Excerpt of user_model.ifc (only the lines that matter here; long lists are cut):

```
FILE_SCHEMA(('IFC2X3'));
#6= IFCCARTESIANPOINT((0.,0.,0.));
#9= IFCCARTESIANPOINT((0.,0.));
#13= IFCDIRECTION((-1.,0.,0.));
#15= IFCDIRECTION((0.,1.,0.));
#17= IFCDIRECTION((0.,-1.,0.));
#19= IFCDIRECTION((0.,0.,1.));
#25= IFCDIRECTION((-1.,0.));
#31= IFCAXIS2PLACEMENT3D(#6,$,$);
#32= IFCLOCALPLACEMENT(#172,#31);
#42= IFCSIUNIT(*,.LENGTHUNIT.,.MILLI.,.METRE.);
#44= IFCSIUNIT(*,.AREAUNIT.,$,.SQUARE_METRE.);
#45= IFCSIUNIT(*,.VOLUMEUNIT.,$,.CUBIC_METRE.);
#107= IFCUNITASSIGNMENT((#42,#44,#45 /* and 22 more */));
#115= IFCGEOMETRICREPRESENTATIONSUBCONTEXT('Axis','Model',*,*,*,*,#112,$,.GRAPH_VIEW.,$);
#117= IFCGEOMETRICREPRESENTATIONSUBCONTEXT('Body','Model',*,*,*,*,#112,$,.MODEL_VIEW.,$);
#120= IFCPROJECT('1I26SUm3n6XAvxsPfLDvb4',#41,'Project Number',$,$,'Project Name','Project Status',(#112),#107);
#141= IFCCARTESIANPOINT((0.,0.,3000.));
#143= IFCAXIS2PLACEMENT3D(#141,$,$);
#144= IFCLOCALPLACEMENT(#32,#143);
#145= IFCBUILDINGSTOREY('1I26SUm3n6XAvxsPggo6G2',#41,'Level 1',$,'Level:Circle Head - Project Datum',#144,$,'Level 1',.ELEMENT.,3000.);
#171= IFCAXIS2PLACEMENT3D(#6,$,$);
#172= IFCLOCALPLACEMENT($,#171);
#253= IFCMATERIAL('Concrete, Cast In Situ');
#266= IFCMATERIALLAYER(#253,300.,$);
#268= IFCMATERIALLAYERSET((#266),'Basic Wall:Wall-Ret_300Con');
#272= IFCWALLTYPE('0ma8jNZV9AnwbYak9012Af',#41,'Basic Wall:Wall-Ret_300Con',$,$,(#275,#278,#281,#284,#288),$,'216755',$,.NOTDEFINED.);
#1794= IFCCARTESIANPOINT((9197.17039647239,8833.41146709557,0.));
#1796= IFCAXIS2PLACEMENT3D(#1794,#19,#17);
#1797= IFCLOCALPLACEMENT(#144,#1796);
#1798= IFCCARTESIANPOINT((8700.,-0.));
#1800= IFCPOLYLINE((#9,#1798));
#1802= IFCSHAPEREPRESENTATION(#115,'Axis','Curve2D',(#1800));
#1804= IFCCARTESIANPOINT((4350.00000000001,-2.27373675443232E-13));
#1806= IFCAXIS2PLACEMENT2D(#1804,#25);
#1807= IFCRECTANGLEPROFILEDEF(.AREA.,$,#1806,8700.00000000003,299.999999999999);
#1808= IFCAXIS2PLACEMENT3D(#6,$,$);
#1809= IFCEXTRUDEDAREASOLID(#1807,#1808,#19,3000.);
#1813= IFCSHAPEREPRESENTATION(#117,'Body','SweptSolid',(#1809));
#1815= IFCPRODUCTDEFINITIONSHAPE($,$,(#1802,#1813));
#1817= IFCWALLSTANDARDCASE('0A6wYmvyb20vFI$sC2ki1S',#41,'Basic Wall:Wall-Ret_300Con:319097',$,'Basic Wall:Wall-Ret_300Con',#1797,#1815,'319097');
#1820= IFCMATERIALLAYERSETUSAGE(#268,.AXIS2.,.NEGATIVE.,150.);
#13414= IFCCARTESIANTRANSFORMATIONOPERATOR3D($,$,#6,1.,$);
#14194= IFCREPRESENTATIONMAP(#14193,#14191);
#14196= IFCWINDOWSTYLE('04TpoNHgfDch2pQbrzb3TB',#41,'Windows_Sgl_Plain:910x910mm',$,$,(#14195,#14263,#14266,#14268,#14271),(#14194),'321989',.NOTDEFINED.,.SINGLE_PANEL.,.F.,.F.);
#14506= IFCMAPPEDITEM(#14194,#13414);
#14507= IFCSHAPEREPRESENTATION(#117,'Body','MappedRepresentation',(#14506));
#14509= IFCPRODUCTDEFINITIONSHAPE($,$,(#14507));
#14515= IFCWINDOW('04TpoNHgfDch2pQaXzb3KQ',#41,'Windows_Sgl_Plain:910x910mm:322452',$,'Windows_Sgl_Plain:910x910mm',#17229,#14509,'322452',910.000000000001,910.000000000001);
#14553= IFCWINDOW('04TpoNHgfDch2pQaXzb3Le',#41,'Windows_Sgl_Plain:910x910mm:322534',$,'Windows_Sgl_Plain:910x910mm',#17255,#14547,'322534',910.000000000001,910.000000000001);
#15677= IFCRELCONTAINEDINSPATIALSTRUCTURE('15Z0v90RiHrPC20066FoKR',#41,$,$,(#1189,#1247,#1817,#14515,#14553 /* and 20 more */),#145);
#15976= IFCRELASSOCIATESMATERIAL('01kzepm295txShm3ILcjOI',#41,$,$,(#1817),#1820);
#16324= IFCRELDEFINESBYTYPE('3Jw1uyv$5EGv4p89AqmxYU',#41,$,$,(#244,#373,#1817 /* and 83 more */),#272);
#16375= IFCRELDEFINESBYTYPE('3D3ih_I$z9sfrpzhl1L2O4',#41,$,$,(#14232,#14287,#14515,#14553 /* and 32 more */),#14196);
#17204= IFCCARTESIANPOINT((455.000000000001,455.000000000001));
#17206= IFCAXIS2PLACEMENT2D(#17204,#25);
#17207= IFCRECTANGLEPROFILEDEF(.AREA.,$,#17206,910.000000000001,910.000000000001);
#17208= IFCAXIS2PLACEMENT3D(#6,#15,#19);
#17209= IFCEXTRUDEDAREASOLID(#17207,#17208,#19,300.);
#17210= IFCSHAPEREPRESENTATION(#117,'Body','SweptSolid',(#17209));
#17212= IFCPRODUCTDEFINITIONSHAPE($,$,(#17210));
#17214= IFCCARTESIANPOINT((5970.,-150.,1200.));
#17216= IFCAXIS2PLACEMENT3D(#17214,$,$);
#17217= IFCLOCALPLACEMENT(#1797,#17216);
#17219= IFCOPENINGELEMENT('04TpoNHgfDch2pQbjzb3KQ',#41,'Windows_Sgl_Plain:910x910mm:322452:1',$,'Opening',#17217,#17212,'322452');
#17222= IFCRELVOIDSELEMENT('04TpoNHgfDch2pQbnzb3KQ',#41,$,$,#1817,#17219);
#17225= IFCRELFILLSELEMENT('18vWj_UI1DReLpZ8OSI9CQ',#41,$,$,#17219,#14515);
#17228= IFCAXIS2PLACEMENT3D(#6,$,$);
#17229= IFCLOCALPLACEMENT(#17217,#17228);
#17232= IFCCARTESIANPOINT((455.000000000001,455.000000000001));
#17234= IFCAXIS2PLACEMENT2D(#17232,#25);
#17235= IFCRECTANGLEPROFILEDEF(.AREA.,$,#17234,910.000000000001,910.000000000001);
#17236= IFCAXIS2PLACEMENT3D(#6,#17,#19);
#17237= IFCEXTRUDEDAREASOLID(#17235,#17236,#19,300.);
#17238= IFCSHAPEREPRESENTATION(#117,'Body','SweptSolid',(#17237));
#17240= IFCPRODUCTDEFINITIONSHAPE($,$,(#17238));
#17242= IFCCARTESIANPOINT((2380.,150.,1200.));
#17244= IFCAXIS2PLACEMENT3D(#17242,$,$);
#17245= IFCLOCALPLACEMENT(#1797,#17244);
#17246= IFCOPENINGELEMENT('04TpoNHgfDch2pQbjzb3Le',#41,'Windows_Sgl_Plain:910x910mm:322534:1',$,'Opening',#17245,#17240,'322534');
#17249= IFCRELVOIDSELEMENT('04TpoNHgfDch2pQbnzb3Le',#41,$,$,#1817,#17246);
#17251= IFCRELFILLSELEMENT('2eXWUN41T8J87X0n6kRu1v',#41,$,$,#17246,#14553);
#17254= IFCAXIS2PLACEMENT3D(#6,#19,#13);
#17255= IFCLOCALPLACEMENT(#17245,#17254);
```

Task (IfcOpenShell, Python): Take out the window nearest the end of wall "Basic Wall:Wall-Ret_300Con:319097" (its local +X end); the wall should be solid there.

```python
import ifcopenshell
import ifcopenshell.api.feature
import ifcopenshell.api.root
import ifcopenshell.geom
import ifcopenshell.util.shape

model = ifcopenshell.open("user_model.ifc")
settings = ifcopenshell.geom.settings()


def volume(element):
    """Net volume in cubic metres, openings subtracted."""
    shape = ifcopenshell.geom.create_shape(settings, element)
    return ifcopenshell.util.shape.get_volume(shape.geometry)


window = model.by_guid("04TpoNHgfDch2pQaXzb3KQ")
opening = window.FillsVoids[0].RelatingOpeningElement
wall = opening.VoidsElements[0].RelatingBuildingElement
before = volume(wall)

ifcopenshell.api.root.remove_product(model, product=window)
ifcopenshell.api.feature.remove_feature(model, feature=opening)

after = volume(wall)

print(f"wall volume {before:.3f} -> {after:.3f} m3")

model.write("user_model_updated.ifc")
```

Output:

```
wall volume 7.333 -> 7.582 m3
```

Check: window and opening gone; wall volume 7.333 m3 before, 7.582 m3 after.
